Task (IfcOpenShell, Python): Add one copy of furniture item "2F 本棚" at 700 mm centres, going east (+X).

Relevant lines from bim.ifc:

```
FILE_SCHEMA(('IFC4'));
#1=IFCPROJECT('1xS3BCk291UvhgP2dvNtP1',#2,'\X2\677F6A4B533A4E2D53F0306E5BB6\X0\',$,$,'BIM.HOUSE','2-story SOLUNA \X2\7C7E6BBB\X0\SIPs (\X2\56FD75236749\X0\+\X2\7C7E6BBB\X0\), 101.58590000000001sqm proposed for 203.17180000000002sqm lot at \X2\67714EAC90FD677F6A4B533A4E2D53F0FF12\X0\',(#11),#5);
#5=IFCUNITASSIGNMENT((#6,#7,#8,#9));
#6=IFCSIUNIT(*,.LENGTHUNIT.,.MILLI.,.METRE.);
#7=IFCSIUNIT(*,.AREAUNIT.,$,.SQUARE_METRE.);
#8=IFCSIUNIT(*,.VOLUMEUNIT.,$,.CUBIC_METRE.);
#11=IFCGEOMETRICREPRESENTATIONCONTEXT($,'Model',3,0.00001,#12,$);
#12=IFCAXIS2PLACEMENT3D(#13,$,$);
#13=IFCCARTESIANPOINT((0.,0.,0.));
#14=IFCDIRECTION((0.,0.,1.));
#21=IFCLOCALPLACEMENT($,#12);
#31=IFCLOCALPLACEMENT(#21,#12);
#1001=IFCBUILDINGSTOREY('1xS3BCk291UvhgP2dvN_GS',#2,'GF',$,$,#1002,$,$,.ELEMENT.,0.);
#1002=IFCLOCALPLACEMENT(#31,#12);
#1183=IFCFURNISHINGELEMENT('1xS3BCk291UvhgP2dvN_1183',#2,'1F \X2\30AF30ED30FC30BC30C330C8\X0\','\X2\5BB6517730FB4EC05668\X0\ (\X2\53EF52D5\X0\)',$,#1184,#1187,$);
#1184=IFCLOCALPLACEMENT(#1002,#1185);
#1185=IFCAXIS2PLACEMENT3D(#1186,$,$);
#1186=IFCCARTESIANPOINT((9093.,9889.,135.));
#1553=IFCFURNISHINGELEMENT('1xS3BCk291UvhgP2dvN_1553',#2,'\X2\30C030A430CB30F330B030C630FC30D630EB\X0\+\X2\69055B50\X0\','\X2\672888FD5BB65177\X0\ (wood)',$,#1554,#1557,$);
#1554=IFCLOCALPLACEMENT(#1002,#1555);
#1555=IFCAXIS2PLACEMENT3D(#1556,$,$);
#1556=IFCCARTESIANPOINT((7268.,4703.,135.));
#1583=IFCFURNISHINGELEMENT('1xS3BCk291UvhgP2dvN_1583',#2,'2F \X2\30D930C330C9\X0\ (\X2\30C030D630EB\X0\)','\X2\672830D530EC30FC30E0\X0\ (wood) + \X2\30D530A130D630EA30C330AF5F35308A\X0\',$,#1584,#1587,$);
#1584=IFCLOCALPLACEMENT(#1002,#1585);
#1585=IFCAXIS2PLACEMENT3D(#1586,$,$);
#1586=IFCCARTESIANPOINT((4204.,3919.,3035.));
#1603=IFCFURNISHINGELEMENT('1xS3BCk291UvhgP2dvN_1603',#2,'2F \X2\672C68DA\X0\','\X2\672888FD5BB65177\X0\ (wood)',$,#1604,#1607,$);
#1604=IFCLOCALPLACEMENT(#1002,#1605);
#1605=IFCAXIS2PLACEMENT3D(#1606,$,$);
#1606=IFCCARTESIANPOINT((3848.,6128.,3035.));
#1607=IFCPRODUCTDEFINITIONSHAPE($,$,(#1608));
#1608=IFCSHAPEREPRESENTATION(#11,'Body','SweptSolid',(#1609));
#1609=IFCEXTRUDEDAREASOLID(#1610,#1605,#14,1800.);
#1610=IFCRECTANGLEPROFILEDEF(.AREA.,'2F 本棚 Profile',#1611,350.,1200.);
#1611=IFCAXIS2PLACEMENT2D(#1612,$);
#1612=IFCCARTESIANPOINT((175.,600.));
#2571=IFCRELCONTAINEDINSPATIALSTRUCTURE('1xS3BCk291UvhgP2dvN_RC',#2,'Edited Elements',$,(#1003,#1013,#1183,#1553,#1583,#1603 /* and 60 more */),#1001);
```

```python
import numpy as np
import ifcopenshell
import ifcopenshell.api.geometry
import ifcopenshell.api.root
import ifcopenshell.util.element
import ifcopenshell.util.placement
import ifcopenshell.util.unit

model = ifcopenshell.open("bim.ifc")
unit_scale = ifcopenshell.util.unit.calculate_unit_scale(model)


def reuse_history(source, copy):
    """copy_class also copies each property set's owner history, people and application; keep the originals."""
    for rel in copy.IsDefinedBy:
        if rel.is_a("IfcRelDefinesByProperties") and (history := rel.RelatingPropertyDefinition.OwnerHistory):
            rel.RelatingPropertyDefinition.OwnerHistory = source.OwnerHistory
            ifcopenshell.util.element.remove_deep2(model, history)


source = model.by_guid("1xS3BCk291UvhgP2dvN_1603")
base = ifcopenshell.util.placement.get_local_placement(source.ObjectPlacement)
step = np.array([1.0, 0.0, 0.0]) * 0.7 / unit_scale

for i in range(1, 2):
    copy = ifcopenshell.api.root.copy_class(model, product=source)
    copy.Representation = ifcopenshell.util.element.copy_deep(
        model, source.Representation, exclude=["IfcGeometricRepresentationContext", "IfcRepresentationMap"]
    )
    reuse_history(source, copy)
    matrix = base.copy()
    matrix[:3, 3] += i * step
    print("added at", matrix[:3, 3].round(3) + 0.0)
    ifcopenshell.api.geometry.edit_object_placement(model, product=copy, matrix=matrix, is_si=False)

model.write("bim-out.ifc")
```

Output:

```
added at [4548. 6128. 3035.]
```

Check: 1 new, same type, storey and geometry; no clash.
